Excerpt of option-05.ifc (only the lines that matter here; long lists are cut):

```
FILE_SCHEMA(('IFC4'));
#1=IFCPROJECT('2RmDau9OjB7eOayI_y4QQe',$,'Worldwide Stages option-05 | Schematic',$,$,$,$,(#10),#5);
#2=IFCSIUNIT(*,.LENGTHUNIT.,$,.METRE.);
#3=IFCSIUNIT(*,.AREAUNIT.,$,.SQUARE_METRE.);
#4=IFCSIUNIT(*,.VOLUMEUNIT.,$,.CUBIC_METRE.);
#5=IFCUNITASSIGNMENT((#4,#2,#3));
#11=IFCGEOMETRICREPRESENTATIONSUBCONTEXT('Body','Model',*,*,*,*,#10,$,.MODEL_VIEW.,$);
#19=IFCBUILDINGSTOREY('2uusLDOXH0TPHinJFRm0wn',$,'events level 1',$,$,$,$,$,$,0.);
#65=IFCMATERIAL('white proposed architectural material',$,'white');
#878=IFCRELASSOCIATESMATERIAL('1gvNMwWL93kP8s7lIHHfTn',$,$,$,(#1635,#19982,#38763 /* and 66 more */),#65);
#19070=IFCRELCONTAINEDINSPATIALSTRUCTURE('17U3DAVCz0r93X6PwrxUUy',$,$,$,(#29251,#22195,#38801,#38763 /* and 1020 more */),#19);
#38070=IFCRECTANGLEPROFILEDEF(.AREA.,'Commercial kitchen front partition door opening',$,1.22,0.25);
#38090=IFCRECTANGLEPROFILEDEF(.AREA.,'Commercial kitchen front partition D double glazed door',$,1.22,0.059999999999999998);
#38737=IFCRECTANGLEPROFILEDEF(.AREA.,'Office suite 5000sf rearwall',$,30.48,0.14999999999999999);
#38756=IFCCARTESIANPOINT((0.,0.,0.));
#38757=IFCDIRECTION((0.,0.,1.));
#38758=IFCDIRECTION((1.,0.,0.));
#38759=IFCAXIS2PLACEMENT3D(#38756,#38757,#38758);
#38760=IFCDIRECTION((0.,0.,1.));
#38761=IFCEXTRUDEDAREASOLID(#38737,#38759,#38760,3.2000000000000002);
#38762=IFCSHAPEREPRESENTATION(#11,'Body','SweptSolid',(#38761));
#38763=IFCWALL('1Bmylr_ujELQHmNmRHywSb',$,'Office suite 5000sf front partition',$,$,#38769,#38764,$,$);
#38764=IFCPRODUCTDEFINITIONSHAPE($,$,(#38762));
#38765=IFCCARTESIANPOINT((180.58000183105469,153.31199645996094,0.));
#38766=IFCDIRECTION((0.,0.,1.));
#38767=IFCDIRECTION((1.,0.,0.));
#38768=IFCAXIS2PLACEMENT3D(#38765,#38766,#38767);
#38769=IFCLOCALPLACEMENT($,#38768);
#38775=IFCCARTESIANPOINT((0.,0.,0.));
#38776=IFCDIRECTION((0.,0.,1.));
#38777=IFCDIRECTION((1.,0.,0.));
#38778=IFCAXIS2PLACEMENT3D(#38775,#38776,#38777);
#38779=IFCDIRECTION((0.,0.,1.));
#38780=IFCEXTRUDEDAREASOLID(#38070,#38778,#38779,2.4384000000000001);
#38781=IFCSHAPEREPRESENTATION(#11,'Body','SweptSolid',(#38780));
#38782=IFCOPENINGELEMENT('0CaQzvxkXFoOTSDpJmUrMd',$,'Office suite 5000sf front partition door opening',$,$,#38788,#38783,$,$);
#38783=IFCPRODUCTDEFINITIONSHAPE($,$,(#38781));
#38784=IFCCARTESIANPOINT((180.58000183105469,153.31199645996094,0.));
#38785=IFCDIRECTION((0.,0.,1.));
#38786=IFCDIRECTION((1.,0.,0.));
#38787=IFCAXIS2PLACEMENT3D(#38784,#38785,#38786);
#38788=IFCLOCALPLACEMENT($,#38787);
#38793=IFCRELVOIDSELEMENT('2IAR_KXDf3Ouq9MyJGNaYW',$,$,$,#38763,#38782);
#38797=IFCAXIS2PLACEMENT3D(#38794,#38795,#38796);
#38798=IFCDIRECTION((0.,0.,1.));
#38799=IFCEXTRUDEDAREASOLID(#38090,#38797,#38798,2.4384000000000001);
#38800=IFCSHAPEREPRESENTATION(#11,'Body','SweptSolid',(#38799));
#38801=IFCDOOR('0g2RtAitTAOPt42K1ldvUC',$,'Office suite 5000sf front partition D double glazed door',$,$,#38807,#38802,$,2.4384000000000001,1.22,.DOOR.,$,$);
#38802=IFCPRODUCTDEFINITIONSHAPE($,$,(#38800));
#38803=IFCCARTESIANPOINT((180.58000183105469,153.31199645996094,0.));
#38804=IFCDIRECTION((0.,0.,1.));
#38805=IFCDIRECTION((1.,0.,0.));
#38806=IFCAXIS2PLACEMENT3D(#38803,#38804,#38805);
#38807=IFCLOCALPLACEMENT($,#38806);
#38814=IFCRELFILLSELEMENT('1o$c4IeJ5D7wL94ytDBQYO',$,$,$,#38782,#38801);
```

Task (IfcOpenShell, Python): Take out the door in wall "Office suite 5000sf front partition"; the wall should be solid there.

```python
import ifcopenshell
import ifcopenshell.api.feature
import ifcopenshell.api.root
import ifcopenshell.geom
import ifcopenshell.util.shape

model = ifcopenshell.open("option-05.ifc")
settings = ifcopenshell.geom.settings()


def volume(element):
    """Net volume in cubic metres, openings subtracted."""
    shape = ifcopenshell.geom.create_shape(settings, element)
    return ifcopenshell.util.shape.get_volume(shape.geometry)


door = model.by_guid("0g2RtAitTAOPt42K1ldvUC")
opening = door.FillsVoids[0].RelatingOpeningElement
wall = opening.VoidsElements[0].RelatingBuildingElement
before = volume(wall)

ifcopenshell.api.root.remove_product(model, product=door)
ifcopenshell.api.feature.remove_feature(model, feature=opening)

after = volume(wall)

print(f"wall volume {before:.3f} -> {after:.3f} m3")

model.write("option-05_updated.ifc")
```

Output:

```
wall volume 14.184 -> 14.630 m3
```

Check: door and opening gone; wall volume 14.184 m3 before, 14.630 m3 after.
